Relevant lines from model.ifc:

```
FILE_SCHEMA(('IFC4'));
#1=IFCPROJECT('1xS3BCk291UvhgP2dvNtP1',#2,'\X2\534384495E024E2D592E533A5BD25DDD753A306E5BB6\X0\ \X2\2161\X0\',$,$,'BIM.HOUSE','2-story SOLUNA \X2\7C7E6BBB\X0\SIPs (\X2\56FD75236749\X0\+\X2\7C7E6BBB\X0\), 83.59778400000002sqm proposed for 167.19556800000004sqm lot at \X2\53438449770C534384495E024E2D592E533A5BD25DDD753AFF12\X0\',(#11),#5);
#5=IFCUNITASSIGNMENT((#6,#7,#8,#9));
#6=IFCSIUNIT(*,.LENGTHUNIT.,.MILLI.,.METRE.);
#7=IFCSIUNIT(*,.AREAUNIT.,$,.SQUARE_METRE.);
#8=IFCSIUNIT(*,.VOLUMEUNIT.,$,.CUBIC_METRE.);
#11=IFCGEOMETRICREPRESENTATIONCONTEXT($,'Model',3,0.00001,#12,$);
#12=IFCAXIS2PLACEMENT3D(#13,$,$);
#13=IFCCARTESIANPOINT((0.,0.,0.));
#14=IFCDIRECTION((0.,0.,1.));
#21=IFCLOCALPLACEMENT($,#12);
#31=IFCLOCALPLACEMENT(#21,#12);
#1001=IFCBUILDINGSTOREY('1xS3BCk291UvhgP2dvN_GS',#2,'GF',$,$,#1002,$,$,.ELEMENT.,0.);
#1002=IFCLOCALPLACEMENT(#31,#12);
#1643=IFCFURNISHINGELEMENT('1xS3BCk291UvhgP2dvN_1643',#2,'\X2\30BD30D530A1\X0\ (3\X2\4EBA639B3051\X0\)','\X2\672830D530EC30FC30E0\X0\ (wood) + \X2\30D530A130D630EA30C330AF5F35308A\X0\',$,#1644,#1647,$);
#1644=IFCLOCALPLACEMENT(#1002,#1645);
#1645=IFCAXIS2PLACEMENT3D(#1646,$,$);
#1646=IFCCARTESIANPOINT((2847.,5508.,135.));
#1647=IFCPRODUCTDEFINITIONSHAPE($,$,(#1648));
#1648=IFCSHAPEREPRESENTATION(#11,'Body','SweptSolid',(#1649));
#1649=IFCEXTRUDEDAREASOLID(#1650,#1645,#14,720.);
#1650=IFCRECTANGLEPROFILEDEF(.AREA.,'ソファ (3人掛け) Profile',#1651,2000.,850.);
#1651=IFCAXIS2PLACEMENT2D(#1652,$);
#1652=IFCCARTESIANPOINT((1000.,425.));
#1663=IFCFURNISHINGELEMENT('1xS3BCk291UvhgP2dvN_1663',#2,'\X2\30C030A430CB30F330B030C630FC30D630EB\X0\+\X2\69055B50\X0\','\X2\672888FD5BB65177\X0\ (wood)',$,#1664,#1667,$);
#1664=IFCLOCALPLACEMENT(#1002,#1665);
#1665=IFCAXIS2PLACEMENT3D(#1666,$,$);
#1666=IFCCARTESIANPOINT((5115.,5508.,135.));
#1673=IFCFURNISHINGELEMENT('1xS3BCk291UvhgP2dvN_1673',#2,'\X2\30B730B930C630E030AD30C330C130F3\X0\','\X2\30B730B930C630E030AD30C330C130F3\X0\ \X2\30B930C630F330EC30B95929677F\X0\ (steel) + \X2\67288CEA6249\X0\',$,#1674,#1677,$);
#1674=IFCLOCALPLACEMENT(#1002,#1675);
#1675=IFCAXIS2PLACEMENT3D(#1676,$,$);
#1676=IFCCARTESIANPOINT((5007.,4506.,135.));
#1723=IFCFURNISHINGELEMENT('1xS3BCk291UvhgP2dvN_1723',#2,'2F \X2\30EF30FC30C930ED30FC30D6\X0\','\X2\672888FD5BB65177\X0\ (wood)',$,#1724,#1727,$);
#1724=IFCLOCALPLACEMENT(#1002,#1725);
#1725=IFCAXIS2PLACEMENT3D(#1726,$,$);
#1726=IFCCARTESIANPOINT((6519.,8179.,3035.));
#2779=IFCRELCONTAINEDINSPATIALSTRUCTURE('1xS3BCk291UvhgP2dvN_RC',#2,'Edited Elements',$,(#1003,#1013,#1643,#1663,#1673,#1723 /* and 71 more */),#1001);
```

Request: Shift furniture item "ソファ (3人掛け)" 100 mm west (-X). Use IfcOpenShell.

```python
import ifcopenshell
import ifcopenshell.api.geometry
import ifcopenshell.util.placement
import ifcopenshell.util.unit

model = ifcopenshell.open("model.ifc")
unit_scale = ifcopenshell.util.unit.calculate_unit_scale(model)

item = model.by_id(1643)
matrix = ifcopenshell.util.placement.get_local_placement(item.ObjectPlacement)
matrix[0, 3] -= 0.1 / unit_scale
ifcopenshell.api.geometry.edit_object_placement(model, product=item, matrix=matrix, is_si=False)

print(ifcopenshell.util.placement.get_local_placement(item.ObjectPlacement).round(3) + 0.0)

model.write("model_updated.ifc")
```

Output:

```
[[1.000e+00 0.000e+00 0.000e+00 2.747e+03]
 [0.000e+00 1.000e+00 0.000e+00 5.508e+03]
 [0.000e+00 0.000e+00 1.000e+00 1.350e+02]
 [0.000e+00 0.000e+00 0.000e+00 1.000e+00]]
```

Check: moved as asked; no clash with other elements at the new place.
